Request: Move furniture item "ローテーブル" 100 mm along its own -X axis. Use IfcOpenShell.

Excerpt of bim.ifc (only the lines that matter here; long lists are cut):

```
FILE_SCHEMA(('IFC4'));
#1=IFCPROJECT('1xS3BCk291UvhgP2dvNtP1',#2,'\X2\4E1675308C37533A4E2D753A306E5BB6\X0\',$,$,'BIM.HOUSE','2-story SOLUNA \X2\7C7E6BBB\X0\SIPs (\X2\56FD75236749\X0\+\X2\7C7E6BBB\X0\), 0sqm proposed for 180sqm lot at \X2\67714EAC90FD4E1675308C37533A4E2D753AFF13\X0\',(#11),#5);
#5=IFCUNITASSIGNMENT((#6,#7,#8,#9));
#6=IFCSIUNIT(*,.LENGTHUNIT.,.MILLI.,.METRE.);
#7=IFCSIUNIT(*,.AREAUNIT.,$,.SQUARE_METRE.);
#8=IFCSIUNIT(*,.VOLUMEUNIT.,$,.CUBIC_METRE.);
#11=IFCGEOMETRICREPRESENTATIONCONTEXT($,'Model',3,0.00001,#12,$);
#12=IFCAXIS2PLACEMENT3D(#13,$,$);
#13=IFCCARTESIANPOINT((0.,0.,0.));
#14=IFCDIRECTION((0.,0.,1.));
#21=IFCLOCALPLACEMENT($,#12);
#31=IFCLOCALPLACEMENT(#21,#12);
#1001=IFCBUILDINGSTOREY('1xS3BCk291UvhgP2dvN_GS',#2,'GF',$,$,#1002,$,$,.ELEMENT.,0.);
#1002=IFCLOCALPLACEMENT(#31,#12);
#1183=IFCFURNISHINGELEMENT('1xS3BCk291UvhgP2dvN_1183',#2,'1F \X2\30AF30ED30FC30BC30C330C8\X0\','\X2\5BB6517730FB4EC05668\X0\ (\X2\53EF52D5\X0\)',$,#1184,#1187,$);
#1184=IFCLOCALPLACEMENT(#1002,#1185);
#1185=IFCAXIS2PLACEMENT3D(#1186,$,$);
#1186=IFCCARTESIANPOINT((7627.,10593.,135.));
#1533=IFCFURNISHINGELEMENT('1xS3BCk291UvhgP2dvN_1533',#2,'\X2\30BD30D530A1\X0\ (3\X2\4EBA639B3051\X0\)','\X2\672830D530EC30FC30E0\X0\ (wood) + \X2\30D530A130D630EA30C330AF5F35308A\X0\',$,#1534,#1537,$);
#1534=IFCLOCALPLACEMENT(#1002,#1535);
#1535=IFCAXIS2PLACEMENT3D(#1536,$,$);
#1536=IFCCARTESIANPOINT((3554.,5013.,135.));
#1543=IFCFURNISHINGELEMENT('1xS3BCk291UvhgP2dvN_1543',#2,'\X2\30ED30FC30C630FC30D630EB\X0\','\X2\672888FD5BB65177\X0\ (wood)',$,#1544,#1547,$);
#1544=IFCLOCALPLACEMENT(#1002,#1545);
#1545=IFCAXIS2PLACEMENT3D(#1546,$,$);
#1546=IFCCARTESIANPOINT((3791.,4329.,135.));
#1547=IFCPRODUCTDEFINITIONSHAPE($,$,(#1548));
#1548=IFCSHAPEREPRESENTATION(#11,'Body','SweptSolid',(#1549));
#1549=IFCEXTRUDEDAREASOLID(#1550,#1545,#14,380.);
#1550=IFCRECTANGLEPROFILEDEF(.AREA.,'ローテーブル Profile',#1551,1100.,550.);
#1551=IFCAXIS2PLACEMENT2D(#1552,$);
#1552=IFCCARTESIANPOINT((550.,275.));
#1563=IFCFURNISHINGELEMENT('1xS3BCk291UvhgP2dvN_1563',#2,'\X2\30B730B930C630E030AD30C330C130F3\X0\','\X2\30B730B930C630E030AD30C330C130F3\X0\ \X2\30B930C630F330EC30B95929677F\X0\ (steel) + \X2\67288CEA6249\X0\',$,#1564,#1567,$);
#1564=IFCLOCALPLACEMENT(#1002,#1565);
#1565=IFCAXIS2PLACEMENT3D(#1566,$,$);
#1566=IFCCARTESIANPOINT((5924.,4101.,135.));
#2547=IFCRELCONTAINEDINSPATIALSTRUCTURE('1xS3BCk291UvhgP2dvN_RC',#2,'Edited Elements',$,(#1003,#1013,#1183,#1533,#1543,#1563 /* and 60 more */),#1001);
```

```python
import ifcopenshell
import ifcopenshell.api.geometry
import ifcopenshell.util.placement

model = ifcopenshell.open("bim.ifc")

item = model.by_id(1543)
matrix = ifcopenshell.util.placement.get_local_placement(item.ObjectPlacement)
matrix[:3, 3] -= matrix[:3, 0] * 100.0
ifcopenshell.api.geometry.edit_object_placement(model, product=item, matrix=matrix, is_si=False)

print(ifcopenshell.util.placement.get_local_placement(item.ObjectPlacement).round(3) + 0.0)

model.write("bim_edited.ifc")
```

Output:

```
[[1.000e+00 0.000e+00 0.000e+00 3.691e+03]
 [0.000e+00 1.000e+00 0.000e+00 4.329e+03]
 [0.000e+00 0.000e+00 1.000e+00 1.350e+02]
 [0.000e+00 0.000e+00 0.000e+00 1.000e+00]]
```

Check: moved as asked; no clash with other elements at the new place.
